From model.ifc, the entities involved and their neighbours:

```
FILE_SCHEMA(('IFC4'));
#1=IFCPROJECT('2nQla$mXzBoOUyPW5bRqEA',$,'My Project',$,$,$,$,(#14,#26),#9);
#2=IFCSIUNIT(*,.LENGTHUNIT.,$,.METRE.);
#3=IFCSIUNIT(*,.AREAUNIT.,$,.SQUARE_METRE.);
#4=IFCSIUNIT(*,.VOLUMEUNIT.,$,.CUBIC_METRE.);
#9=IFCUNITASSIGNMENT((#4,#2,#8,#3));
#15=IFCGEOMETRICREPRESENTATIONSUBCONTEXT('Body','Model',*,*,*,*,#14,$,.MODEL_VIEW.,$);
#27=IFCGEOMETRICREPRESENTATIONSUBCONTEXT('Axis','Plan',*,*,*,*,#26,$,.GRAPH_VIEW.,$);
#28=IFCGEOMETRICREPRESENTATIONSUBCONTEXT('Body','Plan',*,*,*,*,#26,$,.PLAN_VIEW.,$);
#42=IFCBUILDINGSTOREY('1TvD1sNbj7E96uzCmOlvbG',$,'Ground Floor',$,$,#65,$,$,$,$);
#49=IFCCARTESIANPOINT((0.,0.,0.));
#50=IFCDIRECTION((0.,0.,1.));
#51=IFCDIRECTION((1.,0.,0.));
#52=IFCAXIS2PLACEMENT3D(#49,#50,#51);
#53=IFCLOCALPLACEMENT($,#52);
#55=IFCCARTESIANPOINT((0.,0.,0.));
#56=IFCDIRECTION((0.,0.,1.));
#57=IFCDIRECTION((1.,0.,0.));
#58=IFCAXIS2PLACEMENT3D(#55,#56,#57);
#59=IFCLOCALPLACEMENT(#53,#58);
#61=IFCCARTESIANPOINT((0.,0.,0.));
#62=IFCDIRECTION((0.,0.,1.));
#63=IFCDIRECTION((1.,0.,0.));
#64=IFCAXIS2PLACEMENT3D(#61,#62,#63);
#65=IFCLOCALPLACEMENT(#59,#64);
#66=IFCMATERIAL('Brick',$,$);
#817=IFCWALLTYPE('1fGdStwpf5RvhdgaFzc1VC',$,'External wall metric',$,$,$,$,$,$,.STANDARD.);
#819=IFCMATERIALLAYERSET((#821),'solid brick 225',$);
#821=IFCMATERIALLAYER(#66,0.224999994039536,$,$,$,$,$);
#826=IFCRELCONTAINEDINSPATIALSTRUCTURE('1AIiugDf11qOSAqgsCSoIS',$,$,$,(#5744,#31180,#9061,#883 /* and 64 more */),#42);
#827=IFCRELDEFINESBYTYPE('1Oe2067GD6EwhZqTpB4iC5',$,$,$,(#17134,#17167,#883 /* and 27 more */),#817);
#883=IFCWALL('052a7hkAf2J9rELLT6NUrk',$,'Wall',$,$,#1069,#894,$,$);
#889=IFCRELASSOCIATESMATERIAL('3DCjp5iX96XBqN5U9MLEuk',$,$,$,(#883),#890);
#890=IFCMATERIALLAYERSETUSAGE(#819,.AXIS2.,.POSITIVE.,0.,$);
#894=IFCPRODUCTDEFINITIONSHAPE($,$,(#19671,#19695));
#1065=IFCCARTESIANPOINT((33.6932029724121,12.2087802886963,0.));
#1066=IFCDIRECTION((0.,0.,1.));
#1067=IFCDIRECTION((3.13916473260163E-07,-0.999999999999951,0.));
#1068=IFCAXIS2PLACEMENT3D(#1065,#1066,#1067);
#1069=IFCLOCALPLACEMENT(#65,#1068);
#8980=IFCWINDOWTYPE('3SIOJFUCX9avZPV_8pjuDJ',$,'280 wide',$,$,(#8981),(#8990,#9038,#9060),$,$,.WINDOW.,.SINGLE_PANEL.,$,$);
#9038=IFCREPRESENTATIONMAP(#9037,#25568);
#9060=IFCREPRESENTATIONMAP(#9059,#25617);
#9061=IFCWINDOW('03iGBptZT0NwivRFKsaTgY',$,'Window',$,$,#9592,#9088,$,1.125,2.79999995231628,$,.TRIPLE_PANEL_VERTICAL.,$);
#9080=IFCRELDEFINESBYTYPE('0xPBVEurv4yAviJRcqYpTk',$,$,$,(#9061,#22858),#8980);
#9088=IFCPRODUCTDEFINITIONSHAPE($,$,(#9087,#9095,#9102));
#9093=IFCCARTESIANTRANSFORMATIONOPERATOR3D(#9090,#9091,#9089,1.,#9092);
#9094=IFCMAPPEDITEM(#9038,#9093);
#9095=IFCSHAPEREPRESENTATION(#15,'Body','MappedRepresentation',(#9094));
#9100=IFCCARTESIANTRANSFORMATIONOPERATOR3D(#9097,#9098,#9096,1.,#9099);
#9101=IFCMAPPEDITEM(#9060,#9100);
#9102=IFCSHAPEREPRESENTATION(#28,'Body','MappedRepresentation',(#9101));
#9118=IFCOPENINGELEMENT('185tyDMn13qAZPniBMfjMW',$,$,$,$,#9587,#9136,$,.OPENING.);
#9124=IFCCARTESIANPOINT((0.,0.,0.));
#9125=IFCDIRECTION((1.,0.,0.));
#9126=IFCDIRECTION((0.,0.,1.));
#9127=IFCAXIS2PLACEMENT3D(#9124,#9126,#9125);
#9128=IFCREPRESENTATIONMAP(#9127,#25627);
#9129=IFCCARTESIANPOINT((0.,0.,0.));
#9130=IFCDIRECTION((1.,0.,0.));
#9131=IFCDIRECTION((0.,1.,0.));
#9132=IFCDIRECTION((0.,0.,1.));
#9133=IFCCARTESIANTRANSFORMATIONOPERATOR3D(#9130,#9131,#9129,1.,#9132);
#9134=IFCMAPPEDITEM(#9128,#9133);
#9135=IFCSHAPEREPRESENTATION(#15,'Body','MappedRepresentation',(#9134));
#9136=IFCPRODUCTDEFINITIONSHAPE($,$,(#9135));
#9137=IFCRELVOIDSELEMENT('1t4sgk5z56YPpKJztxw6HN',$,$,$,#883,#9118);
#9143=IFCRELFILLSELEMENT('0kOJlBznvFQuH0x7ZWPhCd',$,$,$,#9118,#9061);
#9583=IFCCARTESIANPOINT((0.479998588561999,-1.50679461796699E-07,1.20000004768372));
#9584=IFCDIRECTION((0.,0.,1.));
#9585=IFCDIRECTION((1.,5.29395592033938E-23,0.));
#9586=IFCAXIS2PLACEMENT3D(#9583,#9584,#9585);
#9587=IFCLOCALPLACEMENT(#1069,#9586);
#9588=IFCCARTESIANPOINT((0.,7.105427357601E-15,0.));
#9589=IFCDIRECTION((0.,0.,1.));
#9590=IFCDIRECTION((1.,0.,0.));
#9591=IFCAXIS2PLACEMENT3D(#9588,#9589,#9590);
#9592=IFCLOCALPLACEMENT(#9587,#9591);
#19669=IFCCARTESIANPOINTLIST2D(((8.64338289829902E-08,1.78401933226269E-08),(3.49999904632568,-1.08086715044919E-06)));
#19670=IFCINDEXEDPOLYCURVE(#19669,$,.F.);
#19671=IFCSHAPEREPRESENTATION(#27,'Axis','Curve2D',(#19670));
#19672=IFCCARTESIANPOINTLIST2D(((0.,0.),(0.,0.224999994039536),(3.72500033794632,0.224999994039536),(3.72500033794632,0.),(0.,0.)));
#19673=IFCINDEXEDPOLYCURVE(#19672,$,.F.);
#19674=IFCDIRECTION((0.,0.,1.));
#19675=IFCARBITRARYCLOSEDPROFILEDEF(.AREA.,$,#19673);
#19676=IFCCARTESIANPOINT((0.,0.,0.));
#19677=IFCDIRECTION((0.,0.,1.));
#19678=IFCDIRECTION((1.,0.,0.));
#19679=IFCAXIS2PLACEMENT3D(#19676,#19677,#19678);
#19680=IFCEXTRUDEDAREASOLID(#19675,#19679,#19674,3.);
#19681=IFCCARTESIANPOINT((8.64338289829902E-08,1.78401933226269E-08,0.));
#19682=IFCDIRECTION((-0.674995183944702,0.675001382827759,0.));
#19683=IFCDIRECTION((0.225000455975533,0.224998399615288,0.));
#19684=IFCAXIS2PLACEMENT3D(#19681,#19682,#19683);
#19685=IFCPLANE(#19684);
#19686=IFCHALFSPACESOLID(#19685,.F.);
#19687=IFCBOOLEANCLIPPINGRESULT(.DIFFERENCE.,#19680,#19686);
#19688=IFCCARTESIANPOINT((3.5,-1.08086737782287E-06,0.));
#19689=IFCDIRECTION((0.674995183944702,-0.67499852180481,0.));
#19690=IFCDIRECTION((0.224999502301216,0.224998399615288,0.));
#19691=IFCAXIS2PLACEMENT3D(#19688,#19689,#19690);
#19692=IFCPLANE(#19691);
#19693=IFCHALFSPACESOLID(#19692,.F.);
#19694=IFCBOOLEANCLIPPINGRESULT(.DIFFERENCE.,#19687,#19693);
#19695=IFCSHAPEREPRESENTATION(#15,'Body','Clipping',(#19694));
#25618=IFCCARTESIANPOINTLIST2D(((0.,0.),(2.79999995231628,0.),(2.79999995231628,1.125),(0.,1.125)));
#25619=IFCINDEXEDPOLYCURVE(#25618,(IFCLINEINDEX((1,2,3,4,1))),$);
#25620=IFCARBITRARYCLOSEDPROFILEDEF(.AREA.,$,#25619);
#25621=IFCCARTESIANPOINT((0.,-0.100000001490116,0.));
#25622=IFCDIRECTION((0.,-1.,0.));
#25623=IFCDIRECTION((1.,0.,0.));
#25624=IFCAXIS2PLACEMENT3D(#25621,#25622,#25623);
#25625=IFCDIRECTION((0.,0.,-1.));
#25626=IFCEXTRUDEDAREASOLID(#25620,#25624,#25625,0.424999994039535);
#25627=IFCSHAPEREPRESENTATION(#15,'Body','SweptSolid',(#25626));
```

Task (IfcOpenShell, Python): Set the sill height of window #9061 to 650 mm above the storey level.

```python
import numpy as np
import ifcopenshell
import ifcopenshell.api.geometry
import ifcopenshell.geom
import ifcopenshell.util.element
import ifcopenshell.util.placement
import ifcopenshell.util.shape
import ifcopenshell.util.unit

model = ifcopenshell.open("model.ifc")
unit_scale = ifcopenshell.util.unit.calculate_unit_scale(model)

window = model.by_guid("03iGBptZT0NwivRFKsaTgY")
opening = window.FillsVoids[0].RelatingOpeningElement
storey = ifcopenshell.util.element.get_container(window, ifc_class="IfcBuildingStorey")
level = ifcopenshell.util.placement.get_local_placement(storey.ObjectPlacement)[2, 3]

# The opening's origin need not be at the sill, so measure its lowest point.
shape = ifcopenshell.geom.create_shape(ifcopenshell.geom.settings(), opening)
bottom = ifcopenshell.util.shape.get_shape_bottom_elevation(shape, shape.geometry) / unit_scale
dz = level + 0.65 / unit_scale - bottom

shift = np.array([0.0, 0.0, dz])
# The window is placed relative to its opening, so it follows when the opening moves.
matrix = ifcopenshell.util.placement.get_local_placement(opening.ObjectPlacement)
matrix[:3, 3] += shift
ifcopenshell.api.geometry.edit_object_placement(
    model, product=opening, matrix=matrix, is_si=False, should_transform_children=True
)

print(f"moved by {dz * unit_scale:+.3f} m")

model.write("model_v2.ifc")
```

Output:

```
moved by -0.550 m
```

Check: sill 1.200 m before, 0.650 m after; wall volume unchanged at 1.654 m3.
